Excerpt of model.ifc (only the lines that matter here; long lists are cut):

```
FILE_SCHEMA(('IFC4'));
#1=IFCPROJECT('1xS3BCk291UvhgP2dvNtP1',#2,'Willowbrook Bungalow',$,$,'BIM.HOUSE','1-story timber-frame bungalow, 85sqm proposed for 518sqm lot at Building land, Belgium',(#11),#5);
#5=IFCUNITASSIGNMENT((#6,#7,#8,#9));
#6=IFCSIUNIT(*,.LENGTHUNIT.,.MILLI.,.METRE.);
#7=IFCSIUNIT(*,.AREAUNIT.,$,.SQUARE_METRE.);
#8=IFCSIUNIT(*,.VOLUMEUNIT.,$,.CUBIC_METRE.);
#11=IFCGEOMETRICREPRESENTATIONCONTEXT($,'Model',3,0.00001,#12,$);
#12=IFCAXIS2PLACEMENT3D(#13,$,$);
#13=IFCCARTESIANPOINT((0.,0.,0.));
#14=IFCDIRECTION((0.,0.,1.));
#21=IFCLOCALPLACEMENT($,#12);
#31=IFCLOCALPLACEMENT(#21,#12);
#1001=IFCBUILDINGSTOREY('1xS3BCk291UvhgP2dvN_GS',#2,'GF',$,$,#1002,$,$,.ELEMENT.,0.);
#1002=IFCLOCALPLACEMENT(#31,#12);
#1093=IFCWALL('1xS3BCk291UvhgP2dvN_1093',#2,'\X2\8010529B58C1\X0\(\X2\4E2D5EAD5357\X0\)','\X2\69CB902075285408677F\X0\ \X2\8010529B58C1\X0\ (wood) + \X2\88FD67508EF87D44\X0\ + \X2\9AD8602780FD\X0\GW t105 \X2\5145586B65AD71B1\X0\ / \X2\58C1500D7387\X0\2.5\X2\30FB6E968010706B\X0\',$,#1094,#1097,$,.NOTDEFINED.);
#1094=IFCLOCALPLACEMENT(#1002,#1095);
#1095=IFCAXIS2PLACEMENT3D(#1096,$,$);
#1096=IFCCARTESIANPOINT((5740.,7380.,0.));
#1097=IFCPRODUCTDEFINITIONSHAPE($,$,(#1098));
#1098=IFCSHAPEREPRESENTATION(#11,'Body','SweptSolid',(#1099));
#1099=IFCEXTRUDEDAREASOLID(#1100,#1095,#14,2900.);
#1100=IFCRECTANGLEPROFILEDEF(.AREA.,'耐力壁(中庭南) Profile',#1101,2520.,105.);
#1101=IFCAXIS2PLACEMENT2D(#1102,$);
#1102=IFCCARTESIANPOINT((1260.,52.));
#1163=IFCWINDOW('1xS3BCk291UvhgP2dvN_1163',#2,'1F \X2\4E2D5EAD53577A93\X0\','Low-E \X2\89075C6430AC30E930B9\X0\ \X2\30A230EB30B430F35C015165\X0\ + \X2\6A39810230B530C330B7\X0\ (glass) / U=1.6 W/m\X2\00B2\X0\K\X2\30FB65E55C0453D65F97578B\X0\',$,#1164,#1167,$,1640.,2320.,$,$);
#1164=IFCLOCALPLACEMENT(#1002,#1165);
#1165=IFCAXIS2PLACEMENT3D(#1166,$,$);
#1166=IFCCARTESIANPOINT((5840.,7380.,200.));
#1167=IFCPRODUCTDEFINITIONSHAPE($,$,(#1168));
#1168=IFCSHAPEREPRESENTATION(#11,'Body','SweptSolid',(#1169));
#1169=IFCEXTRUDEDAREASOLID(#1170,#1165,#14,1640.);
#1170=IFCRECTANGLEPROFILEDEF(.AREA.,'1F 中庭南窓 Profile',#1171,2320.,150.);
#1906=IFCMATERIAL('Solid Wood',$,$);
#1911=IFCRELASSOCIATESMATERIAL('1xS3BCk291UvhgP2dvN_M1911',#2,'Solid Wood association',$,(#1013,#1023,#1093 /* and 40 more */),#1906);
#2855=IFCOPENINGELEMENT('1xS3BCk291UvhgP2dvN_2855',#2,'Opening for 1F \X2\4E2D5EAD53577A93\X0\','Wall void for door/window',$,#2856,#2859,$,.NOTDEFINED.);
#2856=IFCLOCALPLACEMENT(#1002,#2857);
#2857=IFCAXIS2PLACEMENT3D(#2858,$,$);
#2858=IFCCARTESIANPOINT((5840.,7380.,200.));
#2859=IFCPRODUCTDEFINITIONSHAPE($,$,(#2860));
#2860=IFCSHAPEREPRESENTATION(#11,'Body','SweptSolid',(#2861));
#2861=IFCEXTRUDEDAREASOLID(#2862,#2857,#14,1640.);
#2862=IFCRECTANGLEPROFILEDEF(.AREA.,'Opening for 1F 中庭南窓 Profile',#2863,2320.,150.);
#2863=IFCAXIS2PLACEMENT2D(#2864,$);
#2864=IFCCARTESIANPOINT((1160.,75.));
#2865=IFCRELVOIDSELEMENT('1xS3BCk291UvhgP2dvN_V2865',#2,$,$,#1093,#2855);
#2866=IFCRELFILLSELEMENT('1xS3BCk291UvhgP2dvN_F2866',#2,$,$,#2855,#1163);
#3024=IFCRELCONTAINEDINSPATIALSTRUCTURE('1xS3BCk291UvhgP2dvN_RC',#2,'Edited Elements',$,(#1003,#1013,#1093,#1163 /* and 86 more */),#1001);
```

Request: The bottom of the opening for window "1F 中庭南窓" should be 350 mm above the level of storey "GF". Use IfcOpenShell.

```python
import numpy as np
import ifcopenshell
import ifcopenshell.api.geometry
import ifcopenshell.geom
import ifcopenshell.util.element
import ifcopenshell.util.placement
import ifcopenshell.util.shape
import ifcopenshell.util.unit

model = ifcopenshell.open("model.ifc")
unit_scale = ifcopenshell.util.unit.calculate_unit_scale(model)

window = model.by_guid("1xS3BCk291UvhgP2dvN_1163")
opening = window.FillsVoids[0].RelatingOpeningElement
storey = ifcopenshell.util.element.get_container(window, ifc_class="IfcBuildingStorey")
level = ifcopenshell.util.placement.get_local_placement(storey.ObjectPlacement)[2, 3]

# The opening's origin need not be at the sill, so measure its lowest point.
shape = ifcopenshell.geom.create_shape(ifcopenshell.geom.settings(), opening)
bottom = ifcopenshell.util.shape.get_shape_bottom_elevation(shape, shape.geometry) / unit_scale
dz = level + 0.35 / unit_scale - bottom

shift = np.array([0.0, 0.0, dz])
# The window is not placed relative to its opening, so move both.
for product in (opening, window):
    matrix = ifcopenshell.util.placement.get_local_placement(product.ObjectPlacement)
    matrix[:3, 3] += shift
    ifcopenshell.api.geometry.edit_object_placement(model, product=product, matrix=matrix, is_si=False)

print(f"moved by {dz * unit_scale:+.3f} m")

model.write("model_v2.ifc")
```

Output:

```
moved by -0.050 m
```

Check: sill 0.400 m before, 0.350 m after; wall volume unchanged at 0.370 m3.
